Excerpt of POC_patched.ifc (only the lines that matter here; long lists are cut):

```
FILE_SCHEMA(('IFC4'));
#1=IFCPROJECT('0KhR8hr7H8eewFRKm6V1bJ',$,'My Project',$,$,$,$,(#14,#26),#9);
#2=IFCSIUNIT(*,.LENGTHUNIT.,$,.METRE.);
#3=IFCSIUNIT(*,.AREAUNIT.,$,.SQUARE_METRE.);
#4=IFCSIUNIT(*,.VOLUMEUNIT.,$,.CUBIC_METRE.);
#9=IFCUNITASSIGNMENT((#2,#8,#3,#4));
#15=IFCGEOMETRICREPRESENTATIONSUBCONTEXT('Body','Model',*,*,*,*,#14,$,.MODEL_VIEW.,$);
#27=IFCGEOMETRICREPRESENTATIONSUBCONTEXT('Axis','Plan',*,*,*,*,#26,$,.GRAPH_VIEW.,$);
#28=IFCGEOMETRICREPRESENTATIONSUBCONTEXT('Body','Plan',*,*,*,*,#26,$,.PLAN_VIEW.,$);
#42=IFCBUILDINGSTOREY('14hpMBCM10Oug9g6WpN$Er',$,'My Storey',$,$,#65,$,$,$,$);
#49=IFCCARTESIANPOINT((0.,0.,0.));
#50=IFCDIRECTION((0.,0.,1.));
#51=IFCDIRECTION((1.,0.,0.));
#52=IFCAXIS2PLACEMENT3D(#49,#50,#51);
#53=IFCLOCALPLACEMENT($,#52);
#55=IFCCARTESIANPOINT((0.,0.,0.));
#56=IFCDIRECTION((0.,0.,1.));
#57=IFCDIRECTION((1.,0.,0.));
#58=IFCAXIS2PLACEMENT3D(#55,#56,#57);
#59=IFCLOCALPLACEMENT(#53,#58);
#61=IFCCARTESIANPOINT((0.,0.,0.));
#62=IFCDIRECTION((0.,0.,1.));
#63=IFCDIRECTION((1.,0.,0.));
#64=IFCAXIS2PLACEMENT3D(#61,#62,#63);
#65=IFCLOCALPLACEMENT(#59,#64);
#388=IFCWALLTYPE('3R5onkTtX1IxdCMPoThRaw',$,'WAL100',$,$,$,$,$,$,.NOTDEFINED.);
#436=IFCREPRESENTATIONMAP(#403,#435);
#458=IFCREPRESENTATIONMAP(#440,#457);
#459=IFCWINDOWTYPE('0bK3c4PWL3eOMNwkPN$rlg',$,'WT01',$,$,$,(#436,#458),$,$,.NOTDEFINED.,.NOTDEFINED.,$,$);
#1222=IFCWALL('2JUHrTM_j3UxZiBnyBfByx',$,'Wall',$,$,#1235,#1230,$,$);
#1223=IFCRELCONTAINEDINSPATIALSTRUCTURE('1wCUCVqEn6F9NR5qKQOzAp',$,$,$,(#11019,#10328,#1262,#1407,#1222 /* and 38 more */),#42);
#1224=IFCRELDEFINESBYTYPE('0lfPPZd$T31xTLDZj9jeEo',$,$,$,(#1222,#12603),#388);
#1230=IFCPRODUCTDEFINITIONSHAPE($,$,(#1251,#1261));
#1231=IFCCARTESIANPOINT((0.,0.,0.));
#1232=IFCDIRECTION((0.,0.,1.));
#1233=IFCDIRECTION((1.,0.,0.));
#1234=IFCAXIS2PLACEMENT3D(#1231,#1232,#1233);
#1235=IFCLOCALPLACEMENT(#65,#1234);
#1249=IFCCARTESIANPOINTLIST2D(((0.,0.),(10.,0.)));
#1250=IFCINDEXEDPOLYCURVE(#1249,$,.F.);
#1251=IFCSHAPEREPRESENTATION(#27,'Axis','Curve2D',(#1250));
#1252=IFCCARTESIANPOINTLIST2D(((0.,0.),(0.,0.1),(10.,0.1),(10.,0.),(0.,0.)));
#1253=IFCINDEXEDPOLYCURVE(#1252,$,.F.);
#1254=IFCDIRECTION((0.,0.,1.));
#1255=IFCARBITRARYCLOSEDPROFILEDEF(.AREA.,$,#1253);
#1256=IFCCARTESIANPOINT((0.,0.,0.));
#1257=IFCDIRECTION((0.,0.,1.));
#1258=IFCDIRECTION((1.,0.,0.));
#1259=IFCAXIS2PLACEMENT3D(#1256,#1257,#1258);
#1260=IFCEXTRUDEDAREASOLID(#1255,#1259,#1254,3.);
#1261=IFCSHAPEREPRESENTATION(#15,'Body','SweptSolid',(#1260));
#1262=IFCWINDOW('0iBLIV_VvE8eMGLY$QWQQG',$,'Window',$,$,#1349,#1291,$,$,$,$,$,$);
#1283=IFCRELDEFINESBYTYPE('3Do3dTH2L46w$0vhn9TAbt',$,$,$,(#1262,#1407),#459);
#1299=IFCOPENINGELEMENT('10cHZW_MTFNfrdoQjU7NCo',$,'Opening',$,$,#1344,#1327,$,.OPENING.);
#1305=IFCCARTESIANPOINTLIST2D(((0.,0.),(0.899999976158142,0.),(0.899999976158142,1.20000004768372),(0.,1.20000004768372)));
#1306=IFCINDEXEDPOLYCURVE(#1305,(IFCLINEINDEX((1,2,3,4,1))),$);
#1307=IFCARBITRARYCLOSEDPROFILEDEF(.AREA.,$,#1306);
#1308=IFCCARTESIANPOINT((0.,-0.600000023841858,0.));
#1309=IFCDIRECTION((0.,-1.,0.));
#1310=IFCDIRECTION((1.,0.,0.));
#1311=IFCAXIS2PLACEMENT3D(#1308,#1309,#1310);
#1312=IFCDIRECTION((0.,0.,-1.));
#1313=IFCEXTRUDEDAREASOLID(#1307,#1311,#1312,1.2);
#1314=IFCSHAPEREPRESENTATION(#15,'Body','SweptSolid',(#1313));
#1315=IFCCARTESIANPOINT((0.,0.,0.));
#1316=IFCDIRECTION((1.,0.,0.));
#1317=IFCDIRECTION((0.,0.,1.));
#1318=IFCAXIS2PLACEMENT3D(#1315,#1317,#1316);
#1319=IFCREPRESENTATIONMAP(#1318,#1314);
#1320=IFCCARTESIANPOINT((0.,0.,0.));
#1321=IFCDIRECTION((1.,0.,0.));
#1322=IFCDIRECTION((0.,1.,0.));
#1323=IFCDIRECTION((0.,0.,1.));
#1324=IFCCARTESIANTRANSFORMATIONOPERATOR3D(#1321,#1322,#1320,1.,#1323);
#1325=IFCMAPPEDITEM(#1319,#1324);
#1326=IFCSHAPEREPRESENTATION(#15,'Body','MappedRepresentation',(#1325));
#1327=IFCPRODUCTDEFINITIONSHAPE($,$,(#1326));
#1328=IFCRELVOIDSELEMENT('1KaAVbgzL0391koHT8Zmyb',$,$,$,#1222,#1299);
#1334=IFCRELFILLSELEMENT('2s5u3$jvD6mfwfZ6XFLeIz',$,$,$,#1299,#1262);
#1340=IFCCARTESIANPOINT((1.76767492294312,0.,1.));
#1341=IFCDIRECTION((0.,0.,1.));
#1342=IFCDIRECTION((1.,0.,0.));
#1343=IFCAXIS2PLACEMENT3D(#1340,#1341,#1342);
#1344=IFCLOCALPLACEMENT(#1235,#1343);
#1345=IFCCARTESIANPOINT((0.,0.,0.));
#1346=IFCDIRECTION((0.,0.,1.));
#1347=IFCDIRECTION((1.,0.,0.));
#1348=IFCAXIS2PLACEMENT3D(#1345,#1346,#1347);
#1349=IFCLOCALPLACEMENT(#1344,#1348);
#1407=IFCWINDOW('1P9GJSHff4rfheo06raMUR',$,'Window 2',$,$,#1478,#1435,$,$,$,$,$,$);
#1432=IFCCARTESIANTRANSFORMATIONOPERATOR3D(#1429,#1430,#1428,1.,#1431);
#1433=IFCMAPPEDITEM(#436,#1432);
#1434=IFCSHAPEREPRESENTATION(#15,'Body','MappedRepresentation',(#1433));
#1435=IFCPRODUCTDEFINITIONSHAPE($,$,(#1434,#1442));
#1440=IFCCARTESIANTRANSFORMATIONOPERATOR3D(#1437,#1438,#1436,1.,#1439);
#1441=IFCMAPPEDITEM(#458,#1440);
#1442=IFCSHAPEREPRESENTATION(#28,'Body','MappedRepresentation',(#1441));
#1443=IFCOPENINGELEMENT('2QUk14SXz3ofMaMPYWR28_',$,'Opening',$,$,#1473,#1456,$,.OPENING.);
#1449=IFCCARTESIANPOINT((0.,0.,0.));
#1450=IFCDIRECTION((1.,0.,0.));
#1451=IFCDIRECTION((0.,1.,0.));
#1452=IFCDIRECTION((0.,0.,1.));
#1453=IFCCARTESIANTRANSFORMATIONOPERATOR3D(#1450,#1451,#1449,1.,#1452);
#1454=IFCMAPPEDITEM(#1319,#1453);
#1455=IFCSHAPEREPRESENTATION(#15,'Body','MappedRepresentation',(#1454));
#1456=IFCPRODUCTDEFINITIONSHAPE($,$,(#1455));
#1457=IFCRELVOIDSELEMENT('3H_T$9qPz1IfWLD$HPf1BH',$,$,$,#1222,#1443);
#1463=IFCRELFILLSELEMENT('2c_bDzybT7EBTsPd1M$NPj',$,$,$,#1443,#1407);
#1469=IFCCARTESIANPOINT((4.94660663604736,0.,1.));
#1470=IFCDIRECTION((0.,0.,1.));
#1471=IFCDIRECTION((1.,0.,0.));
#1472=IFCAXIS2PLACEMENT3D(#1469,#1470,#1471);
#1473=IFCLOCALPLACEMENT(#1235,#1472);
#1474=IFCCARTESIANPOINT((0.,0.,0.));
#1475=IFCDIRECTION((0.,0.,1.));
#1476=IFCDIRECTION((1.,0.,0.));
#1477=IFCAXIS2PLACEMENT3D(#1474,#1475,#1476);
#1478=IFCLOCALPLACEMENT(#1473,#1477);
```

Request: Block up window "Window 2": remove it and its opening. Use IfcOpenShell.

```python
import ifcopenshell
import ifcopenshell.api.feature
import ifcopenshell.api.root
import ifcopenshell.geom
import ifcopenshell.util.shape

model = ifcopenshell.open("POC_patched.ifc")
settings = ifcopenshell.geom.settings()


def volume(element):
    """Net volume in cubic metres, openings subtracted."""
    shape = ifcopenshell.geom.create_shape(settings, element)
    return ifcopenshell.util.shape.get_volume(shape.geometry)


window = model.by_guid("1P9GJSHff4rfheo06raMUR")
opening = window.FillsVoids[0].RelatingOpeningElement
wall = opening.VoidsElements[0].RelatingBuildingElement
before = volume(wall)

ifcopenshell.api.root.remove_product(model, product=window)
ifcopenshell.api.feature.remove_feature(model, feature=opening)

after = volume(wall)

print(f"wall volume {before:.3f} -> {after:.3f} m3")

model.write("POC_patched_rev.ifc")
```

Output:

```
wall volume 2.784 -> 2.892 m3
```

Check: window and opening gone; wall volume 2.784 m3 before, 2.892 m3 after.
